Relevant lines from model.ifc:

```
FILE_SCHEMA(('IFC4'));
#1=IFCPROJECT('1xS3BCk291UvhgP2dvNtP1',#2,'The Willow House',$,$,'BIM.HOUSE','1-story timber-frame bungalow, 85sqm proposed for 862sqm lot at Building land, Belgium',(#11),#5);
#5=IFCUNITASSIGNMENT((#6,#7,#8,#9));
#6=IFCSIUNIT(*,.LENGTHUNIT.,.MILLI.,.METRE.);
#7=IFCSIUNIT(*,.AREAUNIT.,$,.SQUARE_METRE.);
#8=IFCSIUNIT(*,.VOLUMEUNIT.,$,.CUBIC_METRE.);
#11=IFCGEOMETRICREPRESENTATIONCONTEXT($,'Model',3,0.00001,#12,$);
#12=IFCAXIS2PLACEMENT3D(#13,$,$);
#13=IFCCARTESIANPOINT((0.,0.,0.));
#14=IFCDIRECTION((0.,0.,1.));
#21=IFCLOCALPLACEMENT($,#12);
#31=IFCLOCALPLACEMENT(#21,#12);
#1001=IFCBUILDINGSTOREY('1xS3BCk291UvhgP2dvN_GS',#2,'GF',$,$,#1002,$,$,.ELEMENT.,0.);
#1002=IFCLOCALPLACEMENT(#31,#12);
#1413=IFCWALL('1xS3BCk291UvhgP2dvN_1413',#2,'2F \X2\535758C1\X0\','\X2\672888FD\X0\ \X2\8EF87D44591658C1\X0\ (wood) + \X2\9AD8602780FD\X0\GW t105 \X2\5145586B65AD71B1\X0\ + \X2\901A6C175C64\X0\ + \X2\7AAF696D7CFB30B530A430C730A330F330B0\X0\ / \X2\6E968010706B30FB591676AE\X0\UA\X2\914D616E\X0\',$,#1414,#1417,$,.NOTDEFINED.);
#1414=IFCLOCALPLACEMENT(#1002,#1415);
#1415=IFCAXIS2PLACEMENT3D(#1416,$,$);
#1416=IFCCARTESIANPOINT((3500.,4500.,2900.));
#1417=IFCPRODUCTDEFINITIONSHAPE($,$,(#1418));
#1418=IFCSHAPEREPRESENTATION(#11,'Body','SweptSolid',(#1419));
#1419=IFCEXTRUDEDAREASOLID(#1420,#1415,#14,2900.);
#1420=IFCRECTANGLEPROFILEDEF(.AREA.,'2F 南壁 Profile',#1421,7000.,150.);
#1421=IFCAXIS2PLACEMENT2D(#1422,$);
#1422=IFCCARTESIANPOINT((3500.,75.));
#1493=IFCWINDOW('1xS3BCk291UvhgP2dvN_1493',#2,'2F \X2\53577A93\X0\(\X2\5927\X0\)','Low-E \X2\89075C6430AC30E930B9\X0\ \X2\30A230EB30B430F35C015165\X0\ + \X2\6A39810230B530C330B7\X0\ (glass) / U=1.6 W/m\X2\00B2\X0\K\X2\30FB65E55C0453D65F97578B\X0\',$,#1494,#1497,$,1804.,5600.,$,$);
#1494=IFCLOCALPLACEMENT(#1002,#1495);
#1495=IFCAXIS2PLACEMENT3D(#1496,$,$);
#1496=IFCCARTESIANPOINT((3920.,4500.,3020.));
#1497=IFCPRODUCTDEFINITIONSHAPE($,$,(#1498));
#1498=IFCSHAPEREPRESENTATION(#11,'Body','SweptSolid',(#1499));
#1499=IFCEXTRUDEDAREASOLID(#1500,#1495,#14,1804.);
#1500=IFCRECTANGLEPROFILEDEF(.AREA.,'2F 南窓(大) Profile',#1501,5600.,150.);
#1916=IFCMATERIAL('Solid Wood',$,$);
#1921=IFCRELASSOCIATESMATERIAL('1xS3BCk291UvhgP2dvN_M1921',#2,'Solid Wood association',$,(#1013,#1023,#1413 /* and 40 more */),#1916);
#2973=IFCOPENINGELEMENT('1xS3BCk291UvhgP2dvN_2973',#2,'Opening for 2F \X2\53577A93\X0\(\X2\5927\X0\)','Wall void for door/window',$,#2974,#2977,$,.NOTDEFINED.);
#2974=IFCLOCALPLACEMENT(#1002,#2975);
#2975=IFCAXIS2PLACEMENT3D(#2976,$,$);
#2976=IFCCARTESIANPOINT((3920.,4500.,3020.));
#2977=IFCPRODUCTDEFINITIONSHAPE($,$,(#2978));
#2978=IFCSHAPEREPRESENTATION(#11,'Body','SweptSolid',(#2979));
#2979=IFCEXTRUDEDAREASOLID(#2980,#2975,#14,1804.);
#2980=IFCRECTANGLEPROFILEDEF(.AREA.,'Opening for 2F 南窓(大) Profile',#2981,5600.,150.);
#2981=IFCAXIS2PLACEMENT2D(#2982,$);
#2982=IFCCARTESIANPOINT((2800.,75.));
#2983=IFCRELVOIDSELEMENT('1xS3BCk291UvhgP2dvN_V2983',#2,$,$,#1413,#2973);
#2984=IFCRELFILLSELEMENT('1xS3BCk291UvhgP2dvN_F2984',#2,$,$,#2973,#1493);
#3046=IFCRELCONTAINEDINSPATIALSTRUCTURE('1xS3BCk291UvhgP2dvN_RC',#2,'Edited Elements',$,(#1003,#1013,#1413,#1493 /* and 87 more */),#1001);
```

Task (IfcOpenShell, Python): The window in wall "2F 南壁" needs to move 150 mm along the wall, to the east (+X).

```python
import ifcopenshell
import ifcopenshell.api.geometry
import ifcopenshell.util.placement
import ifcopenshell.util.unit

model = ifcopenshell.open("model.ifc")
unit_scale = ifcopenshell.util.unit.calculate_unit_scale(model)

window = model.by_id(1493)
opening = window.FillsVoids[0].RelatingOpeningElement
wall = opening.VoidsElements[0].RelatingBuildingElement

wall_matrix = ifcopenshell.util.placement.get_local_placement(wall.ObjectPlacement)
shift = wall_matrix[:3, 0] * 0.15 / unit_scale
before = ifcopenshell.util.placement.get_local_placement(window.ObjectPlacement)[:3, 3].copy()

# The window is not placed relative to its opening, so move both.
for product in (opening, window):
    matrix = ifcopenshell.util.placement.get_local_placement(product.ObjectPlacement)
    matrix[:3, 3] += shift
    ifcopenshell.api.geometry.edit_object_placement(model, product=product, matrix=matrix, is_si=False)

after = ifcopenshell.util.placement.get_local_placement(window.ObjectPlacement)[:3, 3]
print("window moved by", (after - before).round(3) + 0.0)

model.write("model_updated.ifc")
```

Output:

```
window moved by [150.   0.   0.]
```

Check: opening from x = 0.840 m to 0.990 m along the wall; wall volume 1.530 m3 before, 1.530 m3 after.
